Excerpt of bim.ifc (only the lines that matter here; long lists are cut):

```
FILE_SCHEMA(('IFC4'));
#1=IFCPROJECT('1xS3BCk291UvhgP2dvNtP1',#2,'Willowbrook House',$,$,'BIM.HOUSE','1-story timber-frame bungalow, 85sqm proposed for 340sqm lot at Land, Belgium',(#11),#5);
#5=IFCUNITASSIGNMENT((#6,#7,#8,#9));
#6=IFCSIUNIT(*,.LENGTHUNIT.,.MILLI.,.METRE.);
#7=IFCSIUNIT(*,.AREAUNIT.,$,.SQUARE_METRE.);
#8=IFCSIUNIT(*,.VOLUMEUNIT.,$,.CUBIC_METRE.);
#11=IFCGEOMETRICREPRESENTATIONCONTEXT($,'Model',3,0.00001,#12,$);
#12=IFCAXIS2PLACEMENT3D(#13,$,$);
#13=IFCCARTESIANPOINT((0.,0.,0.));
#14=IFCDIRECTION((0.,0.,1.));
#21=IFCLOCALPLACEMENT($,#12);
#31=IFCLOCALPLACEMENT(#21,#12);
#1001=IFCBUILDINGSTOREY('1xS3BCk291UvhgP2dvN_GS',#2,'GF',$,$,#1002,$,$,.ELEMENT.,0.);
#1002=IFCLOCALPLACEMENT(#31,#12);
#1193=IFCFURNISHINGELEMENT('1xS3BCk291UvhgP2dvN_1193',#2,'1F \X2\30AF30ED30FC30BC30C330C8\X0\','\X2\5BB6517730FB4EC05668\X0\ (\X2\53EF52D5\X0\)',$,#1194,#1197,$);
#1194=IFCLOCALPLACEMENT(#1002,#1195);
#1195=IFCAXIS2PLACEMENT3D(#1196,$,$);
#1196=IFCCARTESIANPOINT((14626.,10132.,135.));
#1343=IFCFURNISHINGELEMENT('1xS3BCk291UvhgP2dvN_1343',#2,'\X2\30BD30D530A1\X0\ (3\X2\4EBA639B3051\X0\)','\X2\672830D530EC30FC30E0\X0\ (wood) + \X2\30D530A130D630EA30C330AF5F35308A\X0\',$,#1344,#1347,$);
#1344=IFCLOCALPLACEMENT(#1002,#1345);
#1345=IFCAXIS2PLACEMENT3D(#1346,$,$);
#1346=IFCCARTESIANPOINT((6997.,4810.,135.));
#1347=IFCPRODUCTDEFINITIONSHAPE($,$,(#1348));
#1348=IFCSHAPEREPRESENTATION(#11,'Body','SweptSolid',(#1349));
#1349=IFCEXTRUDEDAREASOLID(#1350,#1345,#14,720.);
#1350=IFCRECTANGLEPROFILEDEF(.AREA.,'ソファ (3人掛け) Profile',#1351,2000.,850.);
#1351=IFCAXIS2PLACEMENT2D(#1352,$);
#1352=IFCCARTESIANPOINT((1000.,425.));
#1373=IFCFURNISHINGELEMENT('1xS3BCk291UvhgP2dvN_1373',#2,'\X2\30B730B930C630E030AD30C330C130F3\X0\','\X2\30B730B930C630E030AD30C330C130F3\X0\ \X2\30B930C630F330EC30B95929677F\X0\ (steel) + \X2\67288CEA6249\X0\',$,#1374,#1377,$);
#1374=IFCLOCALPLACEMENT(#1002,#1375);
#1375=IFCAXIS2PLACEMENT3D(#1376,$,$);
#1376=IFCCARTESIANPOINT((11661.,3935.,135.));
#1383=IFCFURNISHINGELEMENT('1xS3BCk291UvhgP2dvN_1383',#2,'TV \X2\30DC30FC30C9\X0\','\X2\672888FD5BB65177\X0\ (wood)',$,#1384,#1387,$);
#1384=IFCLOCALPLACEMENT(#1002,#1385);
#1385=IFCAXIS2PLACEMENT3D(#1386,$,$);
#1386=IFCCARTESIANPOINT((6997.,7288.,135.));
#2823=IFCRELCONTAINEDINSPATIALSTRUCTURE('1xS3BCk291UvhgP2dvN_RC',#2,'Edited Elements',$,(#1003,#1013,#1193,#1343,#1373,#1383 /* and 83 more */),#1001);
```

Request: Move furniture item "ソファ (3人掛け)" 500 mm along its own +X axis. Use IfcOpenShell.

```python
import ifcopenshell
import ifcopenshell.api.geometry
import ifcopenshell.util.placement
import ifcopenshell.util.unit

model = ifcopenshell.open("bim.ifc")
unit_scale = ifcopenshell.util.unit.calculate_unit_scale(model)

item = model.by_id(1343)
matrix = ifcopenshell.util.placement.get_local_placement(item.ObjectPlacement)
matrix[:3, 3] += matrix[:3, 0] * 0.5 / unit_scale
ifcopenshell.api.geometry.edit_object_placement(model, product=item, matrix=matrix, is_si=False)

print(ifcopenshell.util.placement.get_local_placement(item.ObjectPlacement).round(3) + 0.0)

model.write("bim_updated.ifc")
```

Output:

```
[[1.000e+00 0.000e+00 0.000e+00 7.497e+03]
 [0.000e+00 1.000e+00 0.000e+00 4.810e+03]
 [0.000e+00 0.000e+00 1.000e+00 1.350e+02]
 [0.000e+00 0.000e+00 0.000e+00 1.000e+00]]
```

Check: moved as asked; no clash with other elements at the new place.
